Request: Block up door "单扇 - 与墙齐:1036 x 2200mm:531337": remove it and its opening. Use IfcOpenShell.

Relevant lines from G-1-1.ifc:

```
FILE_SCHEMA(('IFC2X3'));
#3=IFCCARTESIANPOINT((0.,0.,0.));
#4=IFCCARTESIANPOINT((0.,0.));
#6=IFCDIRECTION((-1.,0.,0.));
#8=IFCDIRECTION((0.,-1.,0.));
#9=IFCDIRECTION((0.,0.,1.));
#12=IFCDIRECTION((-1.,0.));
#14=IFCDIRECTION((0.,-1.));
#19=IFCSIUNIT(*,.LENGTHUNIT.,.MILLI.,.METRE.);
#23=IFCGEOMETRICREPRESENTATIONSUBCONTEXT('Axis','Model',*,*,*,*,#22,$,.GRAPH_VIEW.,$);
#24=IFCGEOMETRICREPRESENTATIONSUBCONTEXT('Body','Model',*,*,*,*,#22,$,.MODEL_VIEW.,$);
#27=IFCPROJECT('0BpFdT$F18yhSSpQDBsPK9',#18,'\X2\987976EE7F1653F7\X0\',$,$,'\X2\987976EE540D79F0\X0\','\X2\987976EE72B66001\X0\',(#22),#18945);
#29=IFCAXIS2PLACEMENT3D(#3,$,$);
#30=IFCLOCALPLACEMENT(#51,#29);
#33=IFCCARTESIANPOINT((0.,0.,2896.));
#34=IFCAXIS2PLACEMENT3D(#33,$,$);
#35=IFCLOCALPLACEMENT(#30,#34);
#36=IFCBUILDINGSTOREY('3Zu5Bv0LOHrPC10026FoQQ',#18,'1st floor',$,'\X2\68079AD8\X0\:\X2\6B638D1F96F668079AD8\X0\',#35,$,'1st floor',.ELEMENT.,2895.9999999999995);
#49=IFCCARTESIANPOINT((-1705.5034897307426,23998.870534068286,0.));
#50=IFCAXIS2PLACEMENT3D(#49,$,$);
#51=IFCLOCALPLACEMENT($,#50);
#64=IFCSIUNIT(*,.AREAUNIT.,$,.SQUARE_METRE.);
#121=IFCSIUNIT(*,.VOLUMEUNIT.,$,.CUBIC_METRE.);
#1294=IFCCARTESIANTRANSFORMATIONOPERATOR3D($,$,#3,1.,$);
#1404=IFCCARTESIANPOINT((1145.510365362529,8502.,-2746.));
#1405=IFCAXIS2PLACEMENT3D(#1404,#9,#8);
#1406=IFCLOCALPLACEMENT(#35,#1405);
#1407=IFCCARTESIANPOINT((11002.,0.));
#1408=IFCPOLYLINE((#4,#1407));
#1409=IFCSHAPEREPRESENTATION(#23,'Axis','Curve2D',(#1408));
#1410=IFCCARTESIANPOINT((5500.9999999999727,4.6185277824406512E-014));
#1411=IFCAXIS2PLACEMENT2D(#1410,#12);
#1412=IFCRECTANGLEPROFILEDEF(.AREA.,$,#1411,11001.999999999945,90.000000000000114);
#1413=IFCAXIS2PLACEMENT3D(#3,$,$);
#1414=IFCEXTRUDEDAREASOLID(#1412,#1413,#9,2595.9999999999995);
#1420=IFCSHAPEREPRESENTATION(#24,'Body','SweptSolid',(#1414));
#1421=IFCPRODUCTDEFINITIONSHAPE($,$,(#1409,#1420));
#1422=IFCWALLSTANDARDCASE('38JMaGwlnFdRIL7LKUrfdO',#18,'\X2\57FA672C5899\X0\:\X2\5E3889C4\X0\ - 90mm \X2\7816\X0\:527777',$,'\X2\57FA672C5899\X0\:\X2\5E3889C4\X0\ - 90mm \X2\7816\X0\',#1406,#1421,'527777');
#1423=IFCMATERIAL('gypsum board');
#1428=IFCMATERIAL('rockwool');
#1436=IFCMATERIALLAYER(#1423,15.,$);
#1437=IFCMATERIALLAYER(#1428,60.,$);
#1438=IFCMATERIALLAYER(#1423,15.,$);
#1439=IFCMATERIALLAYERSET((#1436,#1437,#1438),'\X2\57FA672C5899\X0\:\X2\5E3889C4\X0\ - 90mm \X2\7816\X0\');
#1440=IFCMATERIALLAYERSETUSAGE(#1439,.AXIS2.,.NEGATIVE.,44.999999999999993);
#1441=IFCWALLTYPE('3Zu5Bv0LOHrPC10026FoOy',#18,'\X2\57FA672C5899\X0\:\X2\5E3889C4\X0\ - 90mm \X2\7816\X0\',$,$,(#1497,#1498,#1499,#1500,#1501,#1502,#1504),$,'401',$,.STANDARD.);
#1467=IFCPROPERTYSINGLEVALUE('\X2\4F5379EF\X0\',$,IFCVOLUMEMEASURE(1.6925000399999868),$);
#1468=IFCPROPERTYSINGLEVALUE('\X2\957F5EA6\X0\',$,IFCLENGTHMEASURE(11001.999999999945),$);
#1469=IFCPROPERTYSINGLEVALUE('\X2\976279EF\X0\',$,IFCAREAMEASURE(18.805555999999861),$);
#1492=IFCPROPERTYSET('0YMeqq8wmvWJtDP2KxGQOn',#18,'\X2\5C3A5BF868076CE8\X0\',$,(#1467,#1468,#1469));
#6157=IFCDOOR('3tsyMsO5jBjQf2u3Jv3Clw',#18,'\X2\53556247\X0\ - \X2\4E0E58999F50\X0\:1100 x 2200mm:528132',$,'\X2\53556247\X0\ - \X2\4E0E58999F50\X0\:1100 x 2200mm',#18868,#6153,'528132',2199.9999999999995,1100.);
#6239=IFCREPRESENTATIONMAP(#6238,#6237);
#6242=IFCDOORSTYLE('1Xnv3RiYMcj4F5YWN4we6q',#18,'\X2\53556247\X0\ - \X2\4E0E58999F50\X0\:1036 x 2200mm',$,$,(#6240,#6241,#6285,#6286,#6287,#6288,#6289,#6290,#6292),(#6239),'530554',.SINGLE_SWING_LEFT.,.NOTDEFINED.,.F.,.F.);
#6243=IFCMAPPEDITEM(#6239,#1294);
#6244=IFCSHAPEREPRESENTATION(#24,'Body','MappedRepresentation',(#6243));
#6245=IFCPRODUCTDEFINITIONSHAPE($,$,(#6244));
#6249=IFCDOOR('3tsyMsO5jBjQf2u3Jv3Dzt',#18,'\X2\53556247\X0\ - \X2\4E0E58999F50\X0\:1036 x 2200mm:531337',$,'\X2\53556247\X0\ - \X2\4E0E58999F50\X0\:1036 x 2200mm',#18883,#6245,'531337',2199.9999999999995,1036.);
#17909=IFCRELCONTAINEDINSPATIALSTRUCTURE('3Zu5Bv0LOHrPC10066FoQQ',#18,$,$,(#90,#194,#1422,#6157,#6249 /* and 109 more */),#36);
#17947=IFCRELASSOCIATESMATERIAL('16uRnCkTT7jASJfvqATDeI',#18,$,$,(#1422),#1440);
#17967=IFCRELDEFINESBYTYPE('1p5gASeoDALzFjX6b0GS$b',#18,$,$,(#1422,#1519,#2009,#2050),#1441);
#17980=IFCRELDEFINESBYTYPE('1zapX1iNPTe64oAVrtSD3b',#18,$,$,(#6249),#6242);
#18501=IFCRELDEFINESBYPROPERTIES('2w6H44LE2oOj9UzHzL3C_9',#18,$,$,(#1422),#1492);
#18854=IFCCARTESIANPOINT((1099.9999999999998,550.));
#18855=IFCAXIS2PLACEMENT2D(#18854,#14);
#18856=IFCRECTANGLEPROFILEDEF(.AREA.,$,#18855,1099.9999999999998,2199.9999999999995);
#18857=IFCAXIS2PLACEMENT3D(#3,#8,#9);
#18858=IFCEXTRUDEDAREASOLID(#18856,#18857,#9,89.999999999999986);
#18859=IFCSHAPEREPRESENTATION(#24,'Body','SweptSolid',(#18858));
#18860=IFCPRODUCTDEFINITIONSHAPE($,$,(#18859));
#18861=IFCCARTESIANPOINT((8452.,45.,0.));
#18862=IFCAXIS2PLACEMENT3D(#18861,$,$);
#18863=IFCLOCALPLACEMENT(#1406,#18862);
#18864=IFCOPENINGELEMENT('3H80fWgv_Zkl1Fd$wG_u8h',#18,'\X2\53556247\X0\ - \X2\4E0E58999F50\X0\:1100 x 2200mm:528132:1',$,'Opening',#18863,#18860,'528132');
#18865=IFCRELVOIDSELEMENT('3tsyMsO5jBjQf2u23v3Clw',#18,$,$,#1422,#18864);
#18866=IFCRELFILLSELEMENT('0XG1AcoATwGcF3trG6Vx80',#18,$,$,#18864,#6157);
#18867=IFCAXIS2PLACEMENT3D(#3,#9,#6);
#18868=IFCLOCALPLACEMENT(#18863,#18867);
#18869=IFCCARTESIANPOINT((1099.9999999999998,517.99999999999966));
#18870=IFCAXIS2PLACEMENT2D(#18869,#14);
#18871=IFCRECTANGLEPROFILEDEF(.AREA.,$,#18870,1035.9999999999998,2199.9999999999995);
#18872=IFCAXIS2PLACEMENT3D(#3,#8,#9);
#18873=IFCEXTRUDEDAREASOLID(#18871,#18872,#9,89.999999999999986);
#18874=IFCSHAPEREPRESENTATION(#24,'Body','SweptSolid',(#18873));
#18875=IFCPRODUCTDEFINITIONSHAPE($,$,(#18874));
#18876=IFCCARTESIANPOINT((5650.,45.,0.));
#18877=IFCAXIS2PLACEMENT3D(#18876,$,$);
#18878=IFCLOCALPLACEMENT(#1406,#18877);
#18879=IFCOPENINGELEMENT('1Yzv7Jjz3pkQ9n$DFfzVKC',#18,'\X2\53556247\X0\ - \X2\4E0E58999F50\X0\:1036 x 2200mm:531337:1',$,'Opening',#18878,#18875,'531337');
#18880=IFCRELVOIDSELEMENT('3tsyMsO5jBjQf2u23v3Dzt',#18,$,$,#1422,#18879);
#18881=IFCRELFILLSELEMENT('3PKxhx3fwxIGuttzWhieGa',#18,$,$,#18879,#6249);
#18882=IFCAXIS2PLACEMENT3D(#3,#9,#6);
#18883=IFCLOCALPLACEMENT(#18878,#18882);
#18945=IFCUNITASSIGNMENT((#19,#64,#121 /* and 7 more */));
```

```python
import ifcopenshell
import ifcopenshell.api.feature
import ifcopenshell.api.pset
import ifcopenshell.api.root
import ifcopenshell.geom
import ifcopenshell.util.element
import ifcopenshell.util.shape
import ifcopenshell.util.unit

model = ifcopenshell.open("G-1-1.ifc")
area_scale = ifcopenshell.util.unit.calculate_unit_scale(model, "AREAUNIT")
volume_scale = ifcopenshell.util.unit.calculate_unit_scale(model, "VOLUMEUNIT")
settings = ifcopenshell.geom.settings()


def volume(element):
    """Net volume in cubic metres, openings subtracted."""
    shape = ifcopenshell.geom.create_shape(settings, element)
    return ifcopenshell.util.shape.get_volume(shape.geometry)


door = model.by_id(6249)
opening = door.FillsVoids[0].RelatingOpeningElement
wall = opening.VoidsElements[0].RelatingBuildingElement
before = volume(wall)

ifcopenshell.api.root.remove_product(model, product=door)
ifcopenshell.api.feature.remove_feature(model, feature=opening)

after = volume(wall)
thickness = 0.09  # wall thickness in metres

# Update the wall's stored quantities.
pset = model.by_id(ifcopenshell.util.element.get_pset(wall, "尺寸标注", should_inherit=False)["id"])
ifcopenshell.api.pset.edit_pset(model, pset=pset, properties={
    "体积": model.create_entity("IfcVolumeMeasure", after / volume_scale),
    "面积": model.create_entity("IfcAreaMeasure", after / thickness / area_scale),
})

print(f"wall volume {before:.3f} -> {after:.3f} m3")

model.write("G-1-1-out.ifc")
```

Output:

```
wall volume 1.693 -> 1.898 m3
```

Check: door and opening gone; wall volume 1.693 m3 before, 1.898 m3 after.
